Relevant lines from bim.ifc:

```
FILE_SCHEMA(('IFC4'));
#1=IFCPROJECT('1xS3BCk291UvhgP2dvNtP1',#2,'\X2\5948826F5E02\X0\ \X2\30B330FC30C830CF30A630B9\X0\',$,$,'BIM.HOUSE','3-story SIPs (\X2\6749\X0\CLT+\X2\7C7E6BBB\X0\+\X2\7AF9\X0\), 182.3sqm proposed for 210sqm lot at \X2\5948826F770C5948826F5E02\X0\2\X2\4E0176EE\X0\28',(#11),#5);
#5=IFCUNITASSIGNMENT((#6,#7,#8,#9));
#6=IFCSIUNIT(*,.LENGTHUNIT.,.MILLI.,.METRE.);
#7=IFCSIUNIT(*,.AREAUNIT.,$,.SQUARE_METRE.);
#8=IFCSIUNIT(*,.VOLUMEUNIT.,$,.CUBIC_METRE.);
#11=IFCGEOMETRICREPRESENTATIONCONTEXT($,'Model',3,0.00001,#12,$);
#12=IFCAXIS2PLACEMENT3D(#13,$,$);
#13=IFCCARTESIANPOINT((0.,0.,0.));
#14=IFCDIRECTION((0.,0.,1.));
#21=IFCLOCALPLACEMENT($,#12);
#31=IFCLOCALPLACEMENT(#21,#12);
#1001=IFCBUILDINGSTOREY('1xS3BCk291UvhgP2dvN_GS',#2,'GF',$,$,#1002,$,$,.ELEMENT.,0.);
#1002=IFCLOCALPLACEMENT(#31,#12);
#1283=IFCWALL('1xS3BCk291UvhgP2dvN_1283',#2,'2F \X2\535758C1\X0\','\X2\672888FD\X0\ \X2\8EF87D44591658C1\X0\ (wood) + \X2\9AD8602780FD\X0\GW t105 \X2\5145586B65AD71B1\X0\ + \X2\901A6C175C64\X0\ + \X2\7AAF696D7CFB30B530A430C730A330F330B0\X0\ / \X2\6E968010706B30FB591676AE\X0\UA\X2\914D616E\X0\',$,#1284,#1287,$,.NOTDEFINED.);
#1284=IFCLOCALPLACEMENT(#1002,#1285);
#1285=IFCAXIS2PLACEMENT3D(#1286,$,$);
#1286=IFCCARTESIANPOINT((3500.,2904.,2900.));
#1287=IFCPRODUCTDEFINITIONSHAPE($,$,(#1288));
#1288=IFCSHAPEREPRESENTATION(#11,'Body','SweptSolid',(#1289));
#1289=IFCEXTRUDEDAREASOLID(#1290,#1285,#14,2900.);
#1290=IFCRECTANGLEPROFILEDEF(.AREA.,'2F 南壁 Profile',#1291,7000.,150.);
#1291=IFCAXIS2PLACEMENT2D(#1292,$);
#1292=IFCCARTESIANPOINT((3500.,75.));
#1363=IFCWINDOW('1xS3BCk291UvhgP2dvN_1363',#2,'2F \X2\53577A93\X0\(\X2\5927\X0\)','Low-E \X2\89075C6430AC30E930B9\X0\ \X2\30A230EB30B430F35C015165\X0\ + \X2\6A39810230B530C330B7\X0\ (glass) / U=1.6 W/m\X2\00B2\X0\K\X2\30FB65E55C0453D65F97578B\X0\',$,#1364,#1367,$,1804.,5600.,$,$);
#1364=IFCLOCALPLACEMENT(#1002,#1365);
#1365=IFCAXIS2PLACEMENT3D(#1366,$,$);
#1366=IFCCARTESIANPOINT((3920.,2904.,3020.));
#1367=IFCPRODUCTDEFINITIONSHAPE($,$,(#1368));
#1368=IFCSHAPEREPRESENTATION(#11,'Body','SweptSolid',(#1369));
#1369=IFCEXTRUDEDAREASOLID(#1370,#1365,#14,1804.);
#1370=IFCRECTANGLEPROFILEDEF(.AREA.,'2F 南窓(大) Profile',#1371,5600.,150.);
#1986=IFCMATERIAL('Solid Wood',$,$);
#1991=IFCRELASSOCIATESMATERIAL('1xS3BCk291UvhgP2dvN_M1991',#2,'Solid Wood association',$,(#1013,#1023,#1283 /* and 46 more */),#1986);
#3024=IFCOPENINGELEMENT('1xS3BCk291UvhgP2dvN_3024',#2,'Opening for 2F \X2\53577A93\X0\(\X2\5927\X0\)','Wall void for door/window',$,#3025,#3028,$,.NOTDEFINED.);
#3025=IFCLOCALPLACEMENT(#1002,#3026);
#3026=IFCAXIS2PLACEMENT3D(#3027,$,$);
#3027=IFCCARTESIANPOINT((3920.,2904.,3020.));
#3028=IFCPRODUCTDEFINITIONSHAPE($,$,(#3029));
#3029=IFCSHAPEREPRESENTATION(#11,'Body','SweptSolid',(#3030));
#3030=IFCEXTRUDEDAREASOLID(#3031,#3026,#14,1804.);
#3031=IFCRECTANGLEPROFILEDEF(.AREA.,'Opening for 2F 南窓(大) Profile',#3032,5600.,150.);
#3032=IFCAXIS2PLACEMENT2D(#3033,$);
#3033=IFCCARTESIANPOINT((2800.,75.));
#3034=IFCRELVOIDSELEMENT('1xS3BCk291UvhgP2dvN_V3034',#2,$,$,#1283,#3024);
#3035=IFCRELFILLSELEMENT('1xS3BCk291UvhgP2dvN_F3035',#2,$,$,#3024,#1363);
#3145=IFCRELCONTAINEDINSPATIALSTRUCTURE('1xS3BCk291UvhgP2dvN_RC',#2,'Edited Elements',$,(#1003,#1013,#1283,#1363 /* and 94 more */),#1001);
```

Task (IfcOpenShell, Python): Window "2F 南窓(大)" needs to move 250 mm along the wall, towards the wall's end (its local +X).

```python
import ifcopenshell
import ifcopenshell.api.geometry
import ifcopenshell.util.placement

model = ifcopenshell.open("bim.ifc")

window = model.by_guid("1xS3BCk291UvhgP2dvN_1363")
opening = window.FillsVoids[0].RelatingOpeningElement
wall = opening.VoidsElements[0].RelatingBuildingElement

wall_matrix = ifcopenshell.util.placement.get_local_placement(wall.ObjectPlacement)
shift = wall_matrix[:3, 0] * 250.0
before = ifcopenshell.util.placement.get_local_placement(window.ObjectPlacement)[:3, 3].copy()

# The window is not placed relative to its opening, so move both.
for product in (opening, window):
    matrix = ifcopenshell.util.placement.get_local_placement(product.ObjectPlacement)
    matrix[:3, 3] += shift
    ifcopenshell.api.geometry.edit_object_placement(model, product=product, matrix=matrix, is_si=False)

after = ifcopenshell.util.placement.get_local_placement(window.ObjectPlacement)[:3, 3]
print("window moved by", (after - before).round(3) + 0.0)

model.write("bim_v2.ifc")
```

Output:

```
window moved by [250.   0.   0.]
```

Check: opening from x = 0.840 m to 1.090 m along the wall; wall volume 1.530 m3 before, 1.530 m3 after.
